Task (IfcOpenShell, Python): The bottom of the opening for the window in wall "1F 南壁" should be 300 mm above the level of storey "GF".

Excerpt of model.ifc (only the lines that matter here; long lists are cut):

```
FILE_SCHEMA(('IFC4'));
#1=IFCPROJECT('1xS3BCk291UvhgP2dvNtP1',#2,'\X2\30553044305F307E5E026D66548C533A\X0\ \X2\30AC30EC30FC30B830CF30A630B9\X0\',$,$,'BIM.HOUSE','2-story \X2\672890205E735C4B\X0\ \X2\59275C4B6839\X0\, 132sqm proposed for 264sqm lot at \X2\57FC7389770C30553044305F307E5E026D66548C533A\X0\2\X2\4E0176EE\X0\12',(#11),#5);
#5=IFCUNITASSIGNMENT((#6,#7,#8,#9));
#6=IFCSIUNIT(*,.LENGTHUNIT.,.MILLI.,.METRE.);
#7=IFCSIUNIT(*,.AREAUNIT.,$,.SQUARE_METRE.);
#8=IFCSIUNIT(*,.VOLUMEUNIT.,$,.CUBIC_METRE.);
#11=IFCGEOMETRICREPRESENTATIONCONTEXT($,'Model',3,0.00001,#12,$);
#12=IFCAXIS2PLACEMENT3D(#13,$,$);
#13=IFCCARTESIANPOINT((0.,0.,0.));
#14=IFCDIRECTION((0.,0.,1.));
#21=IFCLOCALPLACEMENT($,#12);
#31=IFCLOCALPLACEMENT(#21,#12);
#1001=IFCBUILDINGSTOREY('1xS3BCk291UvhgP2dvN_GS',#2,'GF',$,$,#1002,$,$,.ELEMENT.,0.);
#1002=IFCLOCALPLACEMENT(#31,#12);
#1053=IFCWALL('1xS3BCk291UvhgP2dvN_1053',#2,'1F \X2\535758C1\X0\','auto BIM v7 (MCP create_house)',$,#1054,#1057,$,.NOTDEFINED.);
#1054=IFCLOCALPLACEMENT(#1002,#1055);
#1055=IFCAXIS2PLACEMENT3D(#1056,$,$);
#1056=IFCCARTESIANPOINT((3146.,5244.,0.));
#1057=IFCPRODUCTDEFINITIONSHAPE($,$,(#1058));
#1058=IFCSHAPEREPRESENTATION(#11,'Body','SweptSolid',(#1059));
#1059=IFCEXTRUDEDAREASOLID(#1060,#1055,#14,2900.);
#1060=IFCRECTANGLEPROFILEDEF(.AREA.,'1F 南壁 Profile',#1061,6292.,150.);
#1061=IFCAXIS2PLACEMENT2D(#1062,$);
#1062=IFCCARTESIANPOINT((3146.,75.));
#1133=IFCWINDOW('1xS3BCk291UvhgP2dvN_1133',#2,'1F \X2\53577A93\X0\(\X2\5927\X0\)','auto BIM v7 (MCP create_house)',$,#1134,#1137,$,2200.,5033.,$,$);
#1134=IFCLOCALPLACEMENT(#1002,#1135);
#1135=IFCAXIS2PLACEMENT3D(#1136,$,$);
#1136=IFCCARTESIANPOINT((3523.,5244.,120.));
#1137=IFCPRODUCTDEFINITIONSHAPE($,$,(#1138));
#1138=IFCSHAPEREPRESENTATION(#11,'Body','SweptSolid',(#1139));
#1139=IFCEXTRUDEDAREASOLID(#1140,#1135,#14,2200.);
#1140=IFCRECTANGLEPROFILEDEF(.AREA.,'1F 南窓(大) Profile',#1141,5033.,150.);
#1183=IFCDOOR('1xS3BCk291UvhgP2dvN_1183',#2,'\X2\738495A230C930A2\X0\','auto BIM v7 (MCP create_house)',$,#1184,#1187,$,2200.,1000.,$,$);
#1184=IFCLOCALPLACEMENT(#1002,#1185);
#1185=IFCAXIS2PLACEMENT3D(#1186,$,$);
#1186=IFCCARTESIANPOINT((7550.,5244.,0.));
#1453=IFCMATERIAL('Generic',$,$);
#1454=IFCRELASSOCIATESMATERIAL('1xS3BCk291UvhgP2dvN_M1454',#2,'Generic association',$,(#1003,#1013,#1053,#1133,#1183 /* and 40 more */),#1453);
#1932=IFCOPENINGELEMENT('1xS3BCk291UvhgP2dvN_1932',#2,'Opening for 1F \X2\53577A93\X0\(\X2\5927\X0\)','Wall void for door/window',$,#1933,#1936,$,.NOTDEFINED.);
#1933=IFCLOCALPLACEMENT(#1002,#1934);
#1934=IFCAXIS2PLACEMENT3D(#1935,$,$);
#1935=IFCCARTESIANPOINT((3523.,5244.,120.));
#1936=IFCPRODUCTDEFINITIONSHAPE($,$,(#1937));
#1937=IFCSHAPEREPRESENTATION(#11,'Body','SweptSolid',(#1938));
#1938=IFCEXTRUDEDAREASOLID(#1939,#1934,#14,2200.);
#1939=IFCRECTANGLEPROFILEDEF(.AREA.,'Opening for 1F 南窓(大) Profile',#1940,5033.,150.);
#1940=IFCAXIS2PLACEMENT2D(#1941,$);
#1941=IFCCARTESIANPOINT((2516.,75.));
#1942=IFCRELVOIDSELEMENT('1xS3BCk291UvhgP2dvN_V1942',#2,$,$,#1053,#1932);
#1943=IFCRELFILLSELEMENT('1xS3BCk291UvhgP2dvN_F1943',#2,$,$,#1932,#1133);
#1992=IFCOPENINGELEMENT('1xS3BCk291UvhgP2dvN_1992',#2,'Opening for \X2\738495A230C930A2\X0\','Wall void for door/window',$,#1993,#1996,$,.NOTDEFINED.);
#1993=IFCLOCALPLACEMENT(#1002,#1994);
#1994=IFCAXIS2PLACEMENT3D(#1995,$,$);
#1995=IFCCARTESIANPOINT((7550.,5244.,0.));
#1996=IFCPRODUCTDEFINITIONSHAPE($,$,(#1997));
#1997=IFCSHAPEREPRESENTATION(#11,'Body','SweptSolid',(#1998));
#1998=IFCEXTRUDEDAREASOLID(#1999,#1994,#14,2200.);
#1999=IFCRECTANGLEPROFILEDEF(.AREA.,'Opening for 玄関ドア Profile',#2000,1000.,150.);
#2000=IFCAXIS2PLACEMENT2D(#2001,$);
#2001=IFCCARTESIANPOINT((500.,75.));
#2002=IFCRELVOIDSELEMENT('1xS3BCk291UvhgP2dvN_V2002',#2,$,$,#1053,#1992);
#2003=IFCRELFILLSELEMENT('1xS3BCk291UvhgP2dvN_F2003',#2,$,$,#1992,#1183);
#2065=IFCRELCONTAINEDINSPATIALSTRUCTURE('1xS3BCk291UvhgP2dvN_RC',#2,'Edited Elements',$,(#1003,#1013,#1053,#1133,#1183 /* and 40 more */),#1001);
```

```python
import numpy as np
import ifcopenshell
import ifcopenshell.api.geometry
import ifcopenshell.geom
import ifcopenshell.util.element
import ifcopenshell.util.placement
import ifcopenshell.util.shape
import ifcopenshell.util.unit

model = ifcopenshell.open("model.ifc")
unit_scale = ifcopenshell.util.unit.calculate_unit_scale(model)

window = model.by_id(1133)
opening = window.FillsVoids[0].RelatingOpeningElement
storey = ifcopenshell.util.element.get_container(window, ifc_class="IfcBuildingStorey")
level = ifcopenshell.util.placement.get_local_placement(storey.ObjectPlacement)[2, 3]

# The opening's origin need not be at the sill, so measure its lowest point.
shape = ifcopenshell.geom.create_shape(ifcopenshell.geom.settings(), opening)
bottom = ifcopenshell.util.shape.get_shape_bottom_elevation(shape, shape.geometry) / unit_scale
dz = level + 0.3 / unit_scale - bottom

shift = np.array([0.0, 0.0, dz])
# The window is not placed relative to its opening, so move both.
for product in (opening, window):
    matrix = ifcopenshell.util.placement.get_local_placement(product.ObjectPlacement)
    matrix[:3, 3] += shift
    ifcopenshell.api.geometry.edit_object_placement(model, product=product, matrix=matrix, is_si=False)

print(f"moved by {dz * unit_scale:+.3f} m")

model.write("model_edited.ifc")
```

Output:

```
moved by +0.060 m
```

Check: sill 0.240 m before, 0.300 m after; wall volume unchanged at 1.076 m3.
